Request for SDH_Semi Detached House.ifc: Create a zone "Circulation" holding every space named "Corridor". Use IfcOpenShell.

First a look at what the model holds.

```python
import ifcopenshell

model = ifcopenshell.open("SDH_Semi Detached House.ifc")
print(model.schema)
seen = {}
for space in model.by_type("IfcSpace"):
    seen[space.LongName] = seen.get(space.LongName, 0) + 1
for name, count in sorted(seen.items(), key=str):
    print(count, "x", name)
print("zones:", [z.Name for z in model.by_type("IfcZone")][:20])
```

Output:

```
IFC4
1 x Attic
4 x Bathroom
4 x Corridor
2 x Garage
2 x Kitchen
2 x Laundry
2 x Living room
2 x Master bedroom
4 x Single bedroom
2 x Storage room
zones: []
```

```python
import ifcopenshell
import ifcopenshell.api.group
import ifcopenshell.api.root

model = ifcopenshell.open("SDH_Semi Detached House.ifc")

names = {"Corridor"}
spaces = [s for s in model.by_type("IfcSpace") if s.LongName in names]

zone = ifcopenshell.api.root.create_entity(model, ifc_class="IfcZone", name="Circulation")
ifcopenshell.api.group.assign_group(model, products=spaces, group=zone)
print(len(spaces), "spaces in", zone.Name)

model.write("SDH_Semi Detached House_v2.ifc")
```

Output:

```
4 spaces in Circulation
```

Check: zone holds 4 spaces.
